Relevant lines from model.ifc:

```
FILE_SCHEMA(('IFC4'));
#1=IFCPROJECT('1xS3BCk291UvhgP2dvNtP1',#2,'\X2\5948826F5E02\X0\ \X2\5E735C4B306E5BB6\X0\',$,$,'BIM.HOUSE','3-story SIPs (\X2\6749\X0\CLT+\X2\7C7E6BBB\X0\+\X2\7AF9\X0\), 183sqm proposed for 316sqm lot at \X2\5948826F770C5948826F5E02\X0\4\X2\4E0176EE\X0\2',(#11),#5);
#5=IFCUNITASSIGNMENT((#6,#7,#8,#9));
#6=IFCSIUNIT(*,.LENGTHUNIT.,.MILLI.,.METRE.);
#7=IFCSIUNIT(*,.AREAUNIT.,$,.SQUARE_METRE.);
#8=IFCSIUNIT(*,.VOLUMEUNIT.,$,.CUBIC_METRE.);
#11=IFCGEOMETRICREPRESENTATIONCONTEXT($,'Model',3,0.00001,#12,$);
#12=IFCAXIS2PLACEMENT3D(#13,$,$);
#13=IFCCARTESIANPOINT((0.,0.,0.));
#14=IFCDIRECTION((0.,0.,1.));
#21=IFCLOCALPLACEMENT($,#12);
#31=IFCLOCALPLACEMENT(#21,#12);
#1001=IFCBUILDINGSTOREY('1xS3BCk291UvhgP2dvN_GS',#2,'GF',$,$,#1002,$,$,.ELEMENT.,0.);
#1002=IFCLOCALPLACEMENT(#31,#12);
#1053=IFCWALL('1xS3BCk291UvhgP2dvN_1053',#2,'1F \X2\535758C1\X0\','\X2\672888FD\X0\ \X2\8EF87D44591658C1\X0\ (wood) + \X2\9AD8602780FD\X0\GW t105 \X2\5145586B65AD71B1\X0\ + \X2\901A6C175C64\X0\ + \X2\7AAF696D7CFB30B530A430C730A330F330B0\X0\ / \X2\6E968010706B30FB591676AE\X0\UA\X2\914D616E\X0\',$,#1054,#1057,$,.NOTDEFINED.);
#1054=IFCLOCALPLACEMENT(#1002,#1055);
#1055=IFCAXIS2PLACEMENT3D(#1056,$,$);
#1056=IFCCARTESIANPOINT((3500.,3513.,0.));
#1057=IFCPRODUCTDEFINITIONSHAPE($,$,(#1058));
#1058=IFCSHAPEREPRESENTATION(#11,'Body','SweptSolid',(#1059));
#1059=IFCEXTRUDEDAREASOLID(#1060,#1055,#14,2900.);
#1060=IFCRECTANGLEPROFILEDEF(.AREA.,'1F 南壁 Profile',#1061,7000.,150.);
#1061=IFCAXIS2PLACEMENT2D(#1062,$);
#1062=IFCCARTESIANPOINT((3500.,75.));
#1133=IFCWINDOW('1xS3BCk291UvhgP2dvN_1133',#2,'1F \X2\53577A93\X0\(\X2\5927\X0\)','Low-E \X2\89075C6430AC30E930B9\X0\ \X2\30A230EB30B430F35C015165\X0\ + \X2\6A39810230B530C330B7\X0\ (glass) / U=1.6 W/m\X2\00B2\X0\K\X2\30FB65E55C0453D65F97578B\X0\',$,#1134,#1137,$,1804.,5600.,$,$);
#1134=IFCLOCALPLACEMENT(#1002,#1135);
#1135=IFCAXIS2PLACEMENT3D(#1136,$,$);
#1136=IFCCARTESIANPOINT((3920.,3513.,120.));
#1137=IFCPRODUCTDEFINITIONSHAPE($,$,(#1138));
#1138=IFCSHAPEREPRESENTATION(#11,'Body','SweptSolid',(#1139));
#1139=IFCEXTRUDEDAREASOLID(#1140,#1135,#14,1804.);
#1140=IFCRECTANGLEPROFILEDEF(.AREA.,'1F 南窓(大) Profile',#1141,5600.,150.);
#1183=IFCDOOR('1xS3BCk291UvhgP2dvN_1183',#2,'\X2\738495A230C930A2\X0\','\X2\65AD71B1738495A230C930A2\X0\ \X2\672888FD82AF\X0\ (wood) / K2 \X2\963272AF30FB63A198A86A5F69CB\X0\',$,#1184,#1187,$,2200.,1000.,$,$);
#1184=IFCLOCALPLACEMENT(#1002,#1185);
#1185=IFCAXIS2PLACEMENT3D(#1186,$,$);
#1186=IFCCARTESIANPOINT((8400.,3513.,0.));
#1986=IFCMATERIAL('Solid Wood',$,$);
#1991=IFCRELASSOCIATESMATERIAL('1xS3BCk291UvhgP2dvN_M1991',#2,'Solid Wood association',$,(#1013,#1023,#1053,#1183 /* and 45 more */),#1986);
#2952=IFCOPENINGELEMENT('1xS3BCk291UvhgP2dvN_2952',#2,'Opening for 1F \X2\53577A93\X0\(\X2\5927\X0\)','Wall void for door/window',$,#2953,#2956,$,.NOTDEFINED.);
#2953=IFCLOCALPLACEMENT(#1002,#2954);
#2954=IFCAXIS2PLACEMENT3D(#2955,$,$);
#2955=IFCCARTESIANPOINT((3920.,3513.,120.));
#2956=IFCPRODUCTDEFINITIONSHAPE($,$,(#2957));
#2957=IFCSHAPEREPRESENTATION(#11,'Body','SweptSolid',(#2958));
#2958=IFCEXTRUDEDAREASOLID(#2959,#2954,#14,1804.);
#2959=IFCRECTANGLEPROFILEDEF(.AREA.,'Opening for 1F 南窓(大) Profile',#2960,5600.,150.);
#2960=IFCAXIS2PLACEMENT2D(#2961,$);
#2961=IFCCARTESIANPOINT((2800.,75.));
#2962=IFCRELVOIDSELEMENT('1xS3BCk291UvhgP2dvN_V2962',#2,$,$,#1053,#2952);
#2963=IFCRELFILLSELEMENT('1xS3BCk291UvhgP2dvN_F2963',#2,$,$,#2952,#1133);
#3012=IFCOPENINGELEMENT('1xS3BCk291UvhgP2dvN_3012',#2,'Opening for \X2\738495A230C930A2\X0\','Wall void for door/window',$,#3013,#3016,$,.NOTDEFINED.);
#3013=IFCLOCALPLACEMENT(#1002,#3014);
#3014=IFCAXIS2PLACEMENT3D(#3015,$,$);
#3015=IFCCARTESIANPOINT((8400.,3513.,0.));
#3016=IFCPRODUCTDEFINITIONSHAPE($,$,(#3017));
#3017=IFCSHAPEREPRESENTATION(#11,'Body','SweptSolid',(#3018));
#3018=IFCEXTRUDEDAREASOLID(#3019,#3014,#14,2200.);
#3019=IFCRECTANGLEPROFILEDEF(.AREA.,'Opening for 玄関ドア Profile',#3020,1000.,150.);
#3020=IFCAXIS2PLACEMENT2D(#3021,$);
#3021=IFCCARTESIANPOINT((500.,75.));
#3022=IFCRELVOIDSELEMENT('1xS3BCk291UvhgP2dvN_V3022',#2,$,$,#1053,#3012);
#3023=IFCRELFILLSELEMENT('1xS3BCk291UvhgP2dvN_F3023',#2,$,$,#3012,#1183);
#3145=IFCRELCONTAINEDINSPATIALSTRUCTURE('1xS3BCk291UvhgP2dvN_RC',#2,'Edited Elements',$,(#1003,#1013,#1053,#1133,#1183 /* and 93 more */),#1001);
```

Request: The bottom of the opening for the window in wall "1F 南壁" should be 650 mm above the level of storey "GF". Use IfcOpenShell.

```python
import numpy as np
import ifcopenshell
import ifcopenshell.api.geometry
import ifcopenshell.geom
import ifcopenshell.util.element
import ifcopenshell.util.placement
import ifcopenshell.util.shape
import ifcopenshell.util.unit

model = ifcopenshell.open("model.ifc")
unit_scale = ifcopenshell.util.unit.calculate_unit_scale(model)

window = model.by_id(1133)
opening = window.FillsVoids[0].RelatingOpeningElement
storey = ifcopenshell.util.element.get_container(window, ifc_class="IfcBuildingStorey")
level = ifcopenshell.util.placement.get_local_placement(storey.ObjectPlacement)[2, 3]

# The opening's origin need not be at the sill, so measure its lowest point.
shape = ifcopenshell.geom.create_shape(ifcopenshell.geom.settings(), opening)
bottom = ifcopenshell.util.shape.get_shape_bottom_elevation(shape, shape.geometry) / unit_scale
dz = level + 0.65 / unit_scale - bottom

shift = np.array([0.0, 0.0, dz])
# The window is not placed relative to its opening, so move both.
for product in (opening, window):
    matrix = ifcopenshell.util.placement.get_local_placement(product.ObjectPlacement)
    matrix[:3, 3] += shift
    ifcopenshell.api.geometry.edit_object_placement(model, product=product, matrix=matrix, is_si=False)

print(f"moved by {dz * unit_scale:+.3f} m")

model.write("model_edited.ifc")
```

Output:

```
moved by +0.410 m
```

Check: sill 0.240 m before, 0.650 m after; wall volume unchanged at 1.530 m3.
